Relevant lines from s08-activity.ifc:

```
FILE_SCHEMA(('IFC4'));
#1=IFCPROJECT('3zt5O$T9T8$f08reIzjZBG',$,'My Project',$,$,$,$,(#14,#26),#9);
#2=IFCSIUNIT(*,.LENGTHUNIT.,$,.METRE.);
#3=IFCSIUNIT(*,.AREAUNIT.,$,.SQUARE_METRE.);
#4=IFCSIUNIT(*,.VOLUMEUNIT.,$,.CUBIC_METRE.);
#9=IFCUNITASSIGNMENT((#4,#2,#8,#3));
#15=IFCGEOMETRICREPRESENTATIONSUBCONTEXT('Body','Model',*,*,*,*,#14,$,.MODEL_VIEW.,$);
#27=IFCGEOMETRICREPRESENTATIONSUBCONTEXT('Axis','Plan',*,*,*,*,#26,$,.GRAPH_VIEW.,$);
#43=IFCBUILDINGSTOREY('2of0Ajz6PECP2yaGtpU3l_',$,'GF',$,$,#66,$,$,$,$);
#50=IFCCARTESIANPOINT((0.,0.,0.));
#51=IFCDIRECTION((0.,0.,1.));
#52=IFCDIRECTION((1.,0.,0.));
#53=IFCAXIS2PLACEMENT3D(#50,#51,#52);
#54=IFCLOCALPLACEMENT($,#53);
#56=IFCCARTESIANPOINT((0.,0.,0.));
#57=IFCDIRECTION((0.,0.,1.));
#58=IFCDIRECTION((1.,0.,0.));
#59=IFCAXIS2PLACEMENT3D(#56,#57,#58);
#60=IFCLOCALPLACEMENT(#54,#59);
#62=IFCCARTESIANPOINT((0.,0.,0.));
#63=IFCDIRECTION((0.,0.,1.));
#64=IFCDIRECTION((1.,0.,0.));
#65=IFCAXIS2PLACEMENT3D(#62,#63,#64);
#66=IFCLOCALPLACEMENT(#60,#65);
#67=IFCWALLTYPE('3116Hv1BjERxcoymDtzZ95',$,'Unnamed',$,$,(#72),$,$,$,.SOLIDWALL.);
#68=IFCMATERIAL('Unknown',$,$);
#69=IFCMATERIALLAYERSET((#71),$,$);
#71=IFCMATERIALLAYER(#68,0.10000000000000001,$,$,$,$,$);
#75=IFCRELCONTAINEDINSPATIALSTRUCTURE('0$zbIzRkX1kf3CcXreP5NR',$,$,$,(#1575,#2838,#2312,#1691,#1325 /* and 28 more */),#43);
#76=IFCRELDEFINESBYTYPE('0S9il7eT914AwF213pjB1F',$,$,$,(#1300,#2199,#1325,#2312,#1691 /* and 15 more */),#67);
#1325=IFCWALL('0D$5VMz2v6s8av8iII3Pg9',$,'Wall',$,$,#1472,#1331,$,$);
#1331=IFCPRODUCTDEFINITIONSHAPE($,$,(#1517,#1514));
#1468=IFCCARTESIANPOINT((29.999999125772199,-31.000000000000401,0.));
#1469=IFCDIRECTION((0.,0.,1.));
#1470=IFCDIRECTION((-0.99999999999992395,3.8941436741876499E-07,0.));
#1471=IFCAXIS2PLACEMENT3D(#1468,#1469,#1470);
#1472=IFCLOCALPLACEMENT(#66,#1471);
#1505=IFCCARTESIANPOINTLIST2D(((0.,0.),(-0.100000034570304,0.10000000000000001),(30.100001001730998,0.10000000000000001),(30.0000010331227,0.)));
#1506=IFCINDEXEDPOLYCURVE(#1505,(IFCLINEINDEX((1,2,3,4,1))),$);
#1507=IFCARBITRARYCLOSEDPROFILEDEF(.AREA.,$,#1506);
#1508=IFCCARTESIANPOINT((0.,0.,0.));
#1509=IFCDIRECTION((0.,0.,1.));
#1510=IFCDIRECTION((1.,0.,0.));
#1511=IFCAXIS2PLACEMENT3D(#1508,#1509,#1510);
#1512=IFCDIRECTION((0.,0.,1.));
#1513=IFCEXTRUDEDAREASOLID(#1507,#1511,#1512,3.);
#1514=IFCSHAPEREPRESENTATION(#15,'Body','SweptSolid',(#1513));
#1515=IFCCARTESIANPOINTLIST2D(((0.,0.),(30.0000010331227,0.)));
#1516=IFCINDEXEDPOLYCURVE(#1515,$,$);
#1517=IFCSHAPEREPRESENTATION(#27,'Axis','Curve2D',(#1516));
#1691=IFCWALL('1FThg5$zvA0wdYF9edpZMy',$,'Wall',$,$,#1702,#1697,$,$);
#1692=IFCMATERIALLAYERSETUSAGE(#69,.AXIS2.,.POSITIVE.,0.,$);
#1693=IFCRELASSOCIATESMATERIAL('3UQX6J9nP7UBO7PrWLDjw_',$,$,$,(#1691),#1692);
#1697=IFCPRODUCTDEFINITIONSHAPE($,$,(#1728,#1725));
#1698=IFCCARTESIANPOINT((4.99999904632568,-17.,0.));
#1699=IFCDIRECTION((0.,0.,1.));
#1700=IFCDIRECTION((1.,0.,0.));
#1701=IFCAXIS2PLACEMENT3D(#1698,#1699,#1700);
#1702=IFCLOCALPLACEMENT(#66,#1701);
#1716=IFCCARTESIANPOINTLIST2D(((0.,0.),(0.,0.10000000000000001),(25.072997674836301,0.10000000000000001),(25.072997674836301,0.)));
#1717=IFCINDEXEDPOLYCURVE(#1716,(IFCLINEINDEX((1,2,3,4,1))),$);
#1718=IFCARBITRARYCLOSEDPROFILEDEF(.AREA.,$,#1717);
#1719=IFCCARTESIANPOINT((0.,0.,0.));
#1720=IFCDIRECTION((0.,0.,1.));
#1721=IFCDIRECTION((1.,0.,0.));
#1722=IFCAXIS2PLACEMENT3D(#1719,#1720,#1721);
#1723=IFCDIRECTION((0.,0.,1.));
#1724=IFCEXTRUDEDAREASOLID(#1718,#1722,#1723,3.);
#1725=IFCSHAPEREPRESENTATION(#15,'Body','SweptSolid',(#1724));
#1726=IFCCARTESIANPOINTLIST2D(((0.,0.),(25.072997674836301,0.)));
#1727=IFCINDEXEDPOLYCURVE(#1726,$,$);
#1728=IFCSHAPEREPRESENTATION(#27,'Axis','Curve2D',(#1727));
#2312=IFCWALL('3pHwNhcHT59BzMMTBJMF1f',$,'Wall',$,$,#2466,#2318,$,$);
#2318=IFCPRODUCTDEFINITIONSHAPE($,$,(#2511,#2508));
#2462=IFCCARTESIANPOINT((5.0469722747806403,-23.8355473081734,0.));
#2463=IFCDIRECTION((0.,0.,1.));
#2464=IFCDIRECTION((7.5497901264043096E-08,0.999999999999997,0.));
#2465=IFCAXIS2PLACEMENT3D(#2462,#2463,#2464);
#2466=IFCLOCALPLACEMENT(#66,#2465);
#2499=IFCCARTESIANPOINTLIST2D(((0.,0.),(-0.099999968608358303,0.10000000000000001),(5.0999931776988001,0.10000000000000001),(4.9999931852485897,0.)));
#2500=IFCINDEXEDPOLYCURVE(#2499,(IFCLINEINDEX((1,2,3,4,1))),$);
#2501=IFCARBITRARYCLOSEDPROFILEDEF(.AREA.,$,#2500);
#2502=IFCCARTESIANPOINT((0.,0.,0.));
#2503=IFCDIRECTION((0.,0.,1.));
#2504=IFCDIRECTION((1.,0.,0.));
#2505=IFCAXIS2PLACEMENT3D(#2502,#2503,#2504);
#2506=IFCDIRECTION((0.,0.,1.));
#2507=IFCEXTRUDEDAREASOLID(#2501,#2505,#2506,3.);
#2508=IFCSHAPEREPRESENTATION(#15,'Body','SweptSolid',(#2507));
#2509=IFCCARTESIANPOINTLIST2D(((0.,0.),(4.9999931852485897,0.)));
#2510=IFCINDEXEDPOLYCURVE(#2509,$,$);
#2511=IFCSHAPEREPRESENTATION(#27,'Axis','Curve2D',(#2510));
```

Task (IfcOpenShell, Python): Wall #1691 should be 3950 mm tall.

```python
import ifcopenshell
import ifcopenshell.geom
import ifcopenshell.util.representation
import ifcopenshell.util.shape
import ifcopenshell.util.unit

model = ifcopenshell.open("s08-activity.ifc")
unit_scale = ifcopenshell.util.unit.calculate_unit_scale(model)
settings = ifcopenshell.geom.settings()


def volume(element):
    """Net volume in cubic metres, openings subtracted."""
    shape = ifcopenshell.geom.create_shape(settings, element)
    return ifcopenshell.util.shape.get_volume(shape.geometry)


wall = model.by_guid("1FThg5$zvA0wdYF9edpZMy")
before = volume(wall)

body = ifcopenshell.util.representation.get_representation(wall, "Model", "Body")
solid = body.Items[0]
old_height = solid.Depth
solid.Depth = 3.95 / unit_scale
after = volume(wall)

print(f"height {old_height:g} -> {solid.Depth:g}, volume {before:.3f} -> {after:.3f} m3")

model.write("s08-activity_updated.ifc")
```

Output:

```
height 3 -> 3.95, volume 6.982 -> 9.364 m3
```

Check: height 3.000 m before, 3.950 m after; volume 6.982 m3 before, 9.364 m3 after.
